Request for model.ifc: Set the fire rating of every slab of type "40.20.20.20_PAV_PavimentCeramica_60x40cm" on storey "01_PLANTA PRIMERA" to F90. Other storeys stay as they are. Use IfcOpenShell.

First a look at what the model holds.

```python
import ifcopenshell
import ifcopenshell.util.element

model = ifcopenshell.open("model.ifc")
print(model.schema)
storey = next(s for s in model.by_type("IfcBuildingStorey") if s.Name == "01_PLANTA PRIMERA")
slabs = [e for e in ifcopenshell.util.element.get_decomposition(storey) if e.is_a("IfcSlab")]
seen = {}
for e in slabs:
    element_type = ifcopenshell.util.element.get_type(e)
    key = (element_type.Name if element_type != e and element_type else None, ifcopenshell.util.element.get_pset(e, "Pset_SlabCommon", "FireRating"))
    seen[key] = seen.get(key, 0) + 1
for (name, value), count in sorted(seen.items(), key=str):
    print(count, "x", name, "|", value)
```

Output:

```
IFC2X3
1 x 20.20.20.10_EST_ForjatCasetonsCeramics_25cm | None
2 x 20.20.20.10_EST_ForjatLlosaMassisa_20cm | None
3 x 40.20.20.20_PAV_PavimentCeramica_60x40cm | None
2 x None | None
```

```python
import ifcopenshell
import ifcopenshell.api.pset
import ifcopenshell.util.element

model = ifcopenshell.open("model.ifc")

storey = next(s for s in model.by_type("IfcBuildingStorey") if s.Name == "01_PLANTA PRIMERA")
slabs = [e for e in ifcopenshell.util.element.get_decomposition(storey) if e.is_a("IfcSlab")]

count = 0
for e in slabs:
    element_type = ifcopenshell.util.element.get_type(e)
    if element_type in (None, e) or element_type.Name != "40.20.20.20_PAV_PavimentCeramica_60x40cm":
        continue
    # add_pset returns the element's existing set when there is one.
    pset = ifcopenshell.api.pset.add_pset(model, product=e, name="Pset_SlabCommon")
    ifcopenshell.api.pset.edit_pset(model, pset=pset, properties={"FireRating": "F90"})
    count += 1

print(count, "slabs updated")

model.write("model_v2.ifc")
```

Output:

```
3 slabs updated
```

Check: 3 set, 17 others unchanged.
